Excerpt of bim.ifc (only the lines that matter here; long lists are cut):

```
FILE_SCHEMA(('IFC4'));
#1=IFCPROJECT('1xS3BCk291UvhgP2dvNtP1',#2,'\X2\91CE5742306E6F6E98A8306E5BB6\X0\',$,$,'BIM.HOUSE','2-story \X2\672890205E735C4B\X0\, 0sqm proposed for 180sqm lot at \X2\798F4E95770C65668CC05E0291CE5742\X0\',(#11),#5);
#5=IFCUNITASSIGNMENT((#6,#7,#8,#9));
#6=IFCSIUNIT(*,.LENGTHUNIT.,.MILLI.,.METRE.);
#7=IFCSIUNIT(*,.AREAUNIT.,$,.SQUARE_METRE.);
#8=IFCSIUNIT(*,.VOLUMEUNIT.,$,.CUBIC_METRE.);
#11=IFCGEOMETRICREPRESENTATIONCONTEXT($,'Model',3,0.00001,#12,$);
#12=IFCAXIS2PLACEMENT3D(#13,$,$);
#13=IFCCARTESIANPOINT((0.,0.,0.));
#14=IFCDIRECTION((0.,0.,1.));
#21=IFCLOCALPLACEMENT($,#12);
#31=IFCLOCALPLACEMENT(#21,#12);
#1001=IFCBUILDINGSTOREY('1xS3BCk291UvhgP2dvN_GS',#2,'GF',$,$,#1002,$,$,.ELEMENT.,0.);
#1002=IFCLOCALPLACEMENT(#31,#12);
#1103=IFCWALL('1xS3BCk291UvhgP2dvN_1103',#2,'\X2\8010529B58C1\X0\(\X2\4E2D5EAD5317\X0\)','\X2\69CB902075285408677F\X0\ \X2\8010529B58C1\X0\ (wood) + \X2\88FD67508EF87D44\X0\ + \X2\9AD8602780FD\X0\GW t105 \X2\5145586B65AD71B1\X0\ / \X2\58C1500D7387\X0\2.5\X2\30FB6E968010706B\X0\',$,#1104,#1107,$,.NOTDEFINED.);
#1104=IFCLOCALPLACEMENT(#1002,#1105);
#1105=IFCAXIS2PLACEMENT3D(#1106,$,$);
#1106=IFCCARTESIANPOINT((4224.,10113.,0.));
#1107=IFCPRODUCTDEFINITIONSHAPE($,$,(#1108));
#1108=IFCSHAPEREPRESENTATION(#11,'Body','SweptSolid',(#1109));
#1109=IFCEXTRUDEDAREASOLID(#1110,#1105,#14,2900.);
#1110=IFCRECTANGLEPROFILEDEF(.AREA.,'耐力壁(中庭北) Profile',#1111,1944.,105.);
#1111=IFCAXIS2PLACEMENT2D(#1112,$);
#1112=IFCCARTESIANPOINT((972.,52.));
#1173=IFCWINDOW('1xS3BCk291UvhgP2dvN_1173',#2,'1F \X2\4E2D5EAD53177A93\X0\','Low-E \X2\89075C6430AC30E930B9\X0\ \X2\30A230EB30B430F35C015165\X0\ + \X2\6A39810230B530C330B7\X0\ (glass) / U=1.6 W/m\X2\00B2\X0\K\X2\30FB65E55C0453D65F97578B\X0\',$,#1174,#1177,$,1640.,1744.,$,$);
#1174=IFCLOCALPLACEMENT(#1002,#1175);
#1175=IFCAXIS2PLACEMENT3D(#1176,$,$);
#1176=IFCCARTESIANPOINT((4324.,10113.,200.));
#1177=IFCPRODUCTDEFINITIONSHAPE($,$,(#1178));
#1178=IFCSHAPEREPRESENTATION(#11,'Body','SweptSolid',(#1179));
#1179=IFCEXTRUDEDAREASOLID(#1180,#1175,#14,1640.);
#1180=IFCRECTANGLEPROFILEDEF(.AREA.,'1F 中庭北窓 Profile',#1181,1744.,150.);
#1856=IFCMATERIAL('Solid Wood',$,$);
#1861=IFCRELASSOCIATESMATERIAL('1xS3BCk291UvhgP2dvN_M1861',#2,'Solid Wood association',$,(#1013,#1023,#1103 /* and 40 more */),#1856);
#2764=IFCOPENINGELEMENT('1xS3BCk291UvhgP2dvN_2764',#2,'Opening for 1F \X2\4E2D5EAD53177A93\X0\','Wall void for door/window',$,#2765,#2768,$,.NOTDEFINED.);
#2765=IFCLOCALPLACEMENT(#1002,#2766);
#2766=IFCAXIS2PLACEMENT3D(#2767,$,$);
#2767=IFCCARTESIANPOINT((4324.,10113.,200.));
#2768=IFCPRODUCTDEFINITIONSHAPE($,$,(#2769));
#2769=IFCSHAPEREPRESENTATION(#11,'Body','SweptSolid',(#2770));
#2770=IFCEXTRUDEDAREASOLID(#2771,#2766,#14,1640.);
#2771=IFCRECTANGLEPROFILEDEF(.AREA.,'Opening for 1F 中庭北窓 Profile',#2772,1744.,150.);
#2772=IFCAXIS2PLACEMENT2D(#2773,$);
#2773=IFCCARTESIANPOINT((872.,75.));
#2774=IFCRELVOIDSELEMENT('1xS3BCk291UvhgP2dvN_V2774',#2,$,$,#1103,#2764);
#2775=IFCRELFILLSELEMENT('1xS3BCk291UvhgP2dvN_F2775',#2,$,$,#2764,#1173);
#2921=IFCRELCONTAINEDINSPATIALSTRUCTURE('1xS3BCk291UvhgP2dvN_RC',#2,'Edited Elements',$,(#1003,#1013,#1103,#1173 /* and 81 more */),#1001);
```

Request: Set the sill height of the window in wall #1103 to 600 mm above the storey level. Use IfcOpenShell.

```python
import numpy as np
import ifcopenshell
import ifcopenshell.api.geometry
import ifcopenshell.geom
import ifcopenshell.util.element
import ifcopenshell.util.placement
import ifcopenshell.util.shape
import ifcopenshell.util.unit

model = ifcopenshell.open("bim.ifc")
unit_scale = ifcopenshell.util.unit.calculate_unit_scale(model)

window = model.by_guid("1xS3BCk291UvhgP2dvN_1173")
opening = window.FillsVoids[0].RelatingOpeningElement
storey = ifcopenshell.util.element.get_container(window, ifc_class="IfcBuildingStorey")
level = ifcopenshell.util.placement.get_local_placement(storey.ObjectPlacement)[2, 3]

# The opening's origin need not be at the sill, so measure its lowest point.
shape = ifcopenshell.geom.create_shape(ifcopenshell.geom.settings(), opening)
bottom = ifcopenshell.util.shape.get_shape_bottom_elevation(shape, shape.geometry) / unit_scale
dz = level + 600.0 - bottom

shift = np.array([0.0, 0.0, dz])
# The window is not placed relative to its opening, so move both.
for product in (opening, window):
    matrix = ifcopenshell.util.placement.get_local_placement(product.ObjectPlacement)
    matrix[:3, 3] += shift
    ifcopenshell.api.geometry.edit_object_placement(model, product=product, matrix=matrix, is_si=False)

print(f"moved by {dz * unit_scale:+.3f} m")

model.write("bim_v2.ifc")
```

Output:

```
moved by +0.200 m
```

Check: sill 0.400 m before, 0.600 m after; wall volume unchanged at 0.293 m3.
